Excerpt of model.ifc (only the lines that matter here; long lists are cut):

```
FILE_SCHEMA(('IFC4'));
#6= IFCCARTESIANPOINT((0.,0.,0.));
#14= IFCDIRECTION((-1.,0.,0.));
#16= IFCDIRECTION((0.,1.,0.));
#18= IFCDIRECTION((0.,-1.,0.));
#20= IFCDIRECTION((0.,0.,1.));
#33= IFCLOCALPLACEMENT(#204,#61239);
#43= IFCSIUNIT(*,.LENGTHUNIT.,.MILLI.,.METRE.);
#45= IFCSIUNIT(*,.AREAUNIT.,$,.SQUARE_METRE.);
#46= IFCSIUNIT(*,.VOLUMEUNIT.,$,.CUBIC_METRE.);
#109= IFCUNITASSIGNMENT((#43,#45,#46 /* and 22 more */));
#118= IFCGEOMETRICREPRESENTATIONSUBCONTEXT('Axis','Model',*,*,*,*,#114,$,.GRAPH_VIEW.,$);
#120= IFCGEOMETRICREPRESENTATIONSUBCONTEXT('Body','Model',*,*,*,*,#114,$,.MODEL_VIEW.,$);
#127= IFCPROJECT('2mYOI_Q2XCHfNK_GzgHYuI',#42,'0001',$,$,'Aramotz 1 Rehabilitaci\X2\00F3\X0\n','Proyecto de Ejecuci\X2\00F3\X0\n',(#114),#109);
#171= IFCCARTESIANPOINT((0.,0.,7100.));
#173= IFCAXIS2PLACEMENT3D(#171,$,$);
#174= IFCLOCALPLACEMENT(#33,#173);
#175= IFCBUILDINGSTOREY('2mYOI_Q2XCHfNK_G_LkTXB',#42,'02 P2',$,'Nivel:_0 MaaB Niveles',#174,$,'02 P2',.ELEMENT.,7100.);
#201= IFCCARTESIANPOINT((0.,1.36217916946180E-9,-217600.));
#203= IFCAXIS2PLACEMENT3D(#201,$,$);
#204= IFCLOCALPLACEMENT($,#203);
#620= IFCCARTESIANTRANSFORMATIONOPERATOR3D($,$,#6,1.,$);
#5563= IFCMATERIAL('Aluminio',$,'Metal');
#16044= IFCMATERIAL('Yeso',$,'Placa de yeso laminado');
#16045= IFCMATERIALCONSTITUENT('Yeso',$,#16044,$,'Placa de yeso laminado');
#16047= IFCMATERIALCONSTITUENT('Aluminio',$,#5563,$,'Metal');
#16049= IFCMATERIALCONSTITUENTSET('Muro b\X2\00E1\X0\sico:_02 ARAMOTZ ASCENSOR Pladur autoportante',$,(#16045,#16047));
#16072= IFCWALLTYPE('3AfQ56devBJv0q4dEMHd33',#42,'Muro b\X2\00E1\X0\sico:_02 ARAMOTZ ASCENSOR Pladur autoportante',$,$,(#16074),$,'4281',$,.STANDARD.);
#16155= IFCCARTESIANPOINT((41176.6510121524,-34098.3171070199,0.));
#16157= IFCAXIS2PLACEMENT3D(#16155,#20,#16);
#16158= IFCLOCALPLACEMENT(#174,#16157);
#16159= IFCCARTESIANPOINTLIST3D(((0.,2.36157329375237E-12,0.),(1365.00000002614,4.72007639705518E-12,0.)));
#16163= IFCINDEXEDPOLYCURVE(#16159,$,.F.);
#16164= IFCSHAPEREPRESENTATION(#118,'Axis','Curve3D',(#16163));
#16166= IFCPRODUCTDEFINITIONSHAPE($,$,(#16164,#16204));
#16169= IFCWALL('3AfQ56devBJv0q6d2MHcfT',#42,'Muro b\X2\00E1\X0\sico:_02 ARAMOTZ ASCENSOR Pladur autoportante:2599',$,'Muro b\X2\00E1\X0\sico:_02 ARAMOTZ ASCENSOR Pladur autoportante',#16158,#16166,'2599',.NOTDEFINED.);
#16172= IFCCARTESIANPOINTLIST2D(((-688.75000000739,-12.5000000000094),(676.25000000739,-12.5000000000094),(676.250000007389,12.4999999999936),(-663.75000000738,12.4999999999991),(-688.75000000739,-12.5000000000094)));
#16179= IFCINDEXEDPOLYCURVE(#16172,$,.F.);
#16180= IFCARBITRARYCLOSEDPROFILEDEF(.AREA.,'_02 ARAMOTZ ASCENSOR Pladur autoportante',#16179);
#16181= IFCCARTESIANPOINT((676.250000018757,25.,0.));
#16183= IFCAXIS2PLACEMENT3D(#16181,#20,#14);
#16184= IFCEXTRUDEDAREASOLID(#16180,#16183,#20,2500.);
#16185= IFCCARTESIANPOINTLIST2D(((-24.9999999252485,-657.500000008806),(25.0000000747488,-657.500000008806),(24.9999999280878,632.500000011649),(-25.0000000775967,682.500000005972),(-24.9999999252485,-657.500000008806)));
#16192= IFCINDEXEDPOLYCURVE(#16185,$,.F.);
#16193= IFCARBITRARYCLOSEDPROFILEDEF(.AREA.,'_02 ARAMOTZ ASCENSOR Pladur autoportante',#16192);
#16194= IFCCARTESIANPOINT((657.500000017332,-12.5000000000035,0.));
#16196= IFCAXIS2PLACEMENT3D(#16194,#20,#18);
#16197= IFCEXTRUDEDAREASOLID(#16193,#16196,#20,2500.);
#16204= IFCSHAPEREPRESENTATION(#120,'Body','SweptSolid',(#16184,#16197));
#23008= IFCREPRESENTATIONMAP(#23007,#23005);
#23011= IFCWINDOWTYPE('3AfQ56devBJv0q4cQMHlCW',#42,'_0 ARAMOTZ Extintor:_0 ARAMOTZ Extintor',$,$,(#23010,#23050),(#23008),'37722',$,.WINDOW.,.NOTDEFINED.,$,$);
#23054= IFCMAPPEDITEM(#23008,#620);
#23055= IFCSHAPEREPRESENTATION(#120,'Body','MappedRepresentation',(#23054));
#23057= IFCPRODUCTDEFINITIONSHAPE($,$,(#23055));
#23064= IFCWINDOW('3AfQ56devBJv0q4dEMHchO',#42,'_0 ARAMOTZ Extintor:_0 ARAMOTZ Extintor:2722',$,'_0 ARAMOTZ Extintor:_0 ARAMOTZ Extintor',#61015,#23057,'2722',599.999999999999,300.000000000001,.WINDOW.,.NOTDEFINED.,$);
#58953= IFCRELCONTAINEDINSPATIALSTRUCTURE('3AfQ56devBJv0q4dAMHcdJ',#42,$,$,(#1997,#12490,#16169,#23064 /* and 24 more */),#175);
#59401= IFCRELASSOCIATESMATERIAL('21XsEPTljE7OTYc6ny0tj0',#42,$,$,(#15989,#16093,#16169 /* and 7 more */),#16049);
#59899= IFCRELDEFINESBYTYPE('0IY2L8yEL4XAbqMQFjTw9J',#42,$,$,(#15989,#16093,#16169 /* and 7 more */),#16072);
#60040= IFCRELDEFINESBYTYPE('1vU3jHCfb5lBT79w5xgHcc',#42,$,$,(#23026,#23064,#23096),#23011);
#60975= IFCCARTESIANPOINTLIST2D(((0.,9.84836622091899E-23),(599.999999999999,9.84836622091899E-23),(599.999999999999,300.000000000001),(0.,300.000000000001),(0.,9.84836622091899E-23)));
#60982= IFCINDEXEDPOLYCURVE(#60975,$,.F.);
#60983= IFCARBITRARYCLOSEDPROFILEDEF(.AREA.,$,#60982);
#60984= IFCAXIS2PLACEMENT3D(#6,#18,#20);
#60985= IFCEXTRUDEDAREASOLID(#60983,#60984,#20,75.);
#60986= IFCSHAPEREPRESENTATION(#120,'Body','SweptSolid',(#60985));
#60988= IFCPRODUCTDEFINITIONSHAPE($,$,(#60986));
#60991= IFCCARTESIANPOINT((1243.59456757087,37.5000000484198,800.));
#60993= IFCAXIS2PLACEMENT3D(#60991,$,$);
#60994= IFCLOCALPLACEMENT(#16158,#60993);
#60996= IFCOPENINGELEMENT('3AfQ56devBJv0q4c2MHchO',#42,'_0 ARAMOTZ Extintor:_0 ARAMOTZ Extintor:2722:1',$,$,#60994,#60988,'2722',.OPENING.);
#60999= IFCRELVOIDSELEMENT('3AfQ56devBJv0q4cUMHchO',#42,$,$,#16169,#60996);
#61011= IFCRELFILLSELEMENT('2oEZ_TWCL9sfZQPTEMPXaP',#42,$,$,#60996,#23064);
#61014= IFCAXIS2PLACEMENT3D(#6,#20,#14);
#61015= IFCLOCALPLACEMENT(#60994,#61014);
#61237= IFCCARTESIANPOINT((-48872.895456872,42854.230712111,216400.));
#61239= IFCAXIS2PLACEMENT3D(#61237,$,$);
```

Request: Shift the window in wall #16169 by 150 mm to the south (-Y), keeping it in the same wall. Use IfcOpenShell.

```python
import ifcopenshell
import ifcopenshell.api.geometry
import ifcopenshell.util.placement

model = ifcopenshell.open("model.ifc")

window = model.by_id(23064)
opening = window.FillsVoids[0].RelatingOpeningElement
wall = opening.VoidsElements[0].RelatingBuildingElement

wall_matrix = ifcopenshell.util.placement.get_local_placement(wall.ObjectPlacement)
shift = wall_matrix[:3, 0] * -150.0
before = ifcopenshell.util.placement.get_local_placement(window.ObjectPlacement)[:3, 3].copy()

# The window is placed relative to its opening, so it follows when the opening moves.
matrix = ifcopenshell.util.placement.get_local_placement(opening.ObjectPlacement)
matrix[:3, 3] += shift
ifcopenshell.api.geometry.edit_object_placement(
    model, product=opening, matrix=matrix, is_si=False, should_transform_children=True
)

after = ifcopenshell.util.placement.get_local_placement(window.ObjectPlacement)[:3, 3]
print("window moved by", (after - before).round(3) + 0.0)

model.write("model_rev.ifc")
```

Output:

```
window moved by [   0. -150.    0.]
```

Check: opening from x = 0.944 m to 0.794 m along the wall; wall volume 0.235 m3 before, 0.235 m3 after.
